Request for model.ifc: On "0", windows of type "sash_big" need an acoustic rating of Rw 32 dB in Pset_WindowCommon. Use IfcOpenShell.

First a look at what the model holds.

```python
import ifcopenshell
import ifcopenshell.util.element

model = ifcopenshell.open("model.ifc")
print(model.schema)
storey = next(s for s in model.by_type("IfcBuildingStorey") if s.Name == "0")
windows = [e for e in ifcopenshell.util.element.get_decomposition(storey) if e.is_a("IfcWindow")]
seen = {}
for e in windows:
    element_type = ifcopenshell.util.element.get_type(e)
    key = (element_type.Name if element_type != e and element_type else None, ifcopenshell.util.element.get_pset(e, "Pset_WindowCommon", "AcousticRating"))
    seen[key] = seen.get(key, 0) + 1
for (name, value), count in sorted(seen.items(), key=str):
    print(count, "x", name, "|", value)
```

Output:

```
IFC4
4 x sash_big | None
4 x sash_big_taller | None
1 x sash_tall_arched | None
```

```python
import ifcopenshell
import ifcopenshell.api.pset
import ifcopenshell.util.element

model = ifcopenshell.open("model.ifc")

storey = next(s for s in model.by_type("IfcBuildingStorey") if s.Name == "0")
windows = [e for e in ifcopenshell.util.element.get_decomposition(storey) if e.is_a("IfcWindow")]

count = 0
for e in windows:
    element_type = ifcopenshell.util.element.get_type(e)
    if element_type in (None, e) or element_type.Name != "sash_big":
        continue
    # add_pset returns the element's existing set when there is one.
    pset = ifcopenshell.api.pset.add_pset(model, product=e, name="Pset_WindowCommon")
    ifcopenshell.api.pset.edit_pset(model, pset=pset, properties={"AcousticRating": "Rw 32 dB"})
    count += 1

print(count, "windows updated")

model.write("model_edited.ifc")
```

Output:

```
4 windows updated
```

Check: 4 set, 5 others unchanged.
